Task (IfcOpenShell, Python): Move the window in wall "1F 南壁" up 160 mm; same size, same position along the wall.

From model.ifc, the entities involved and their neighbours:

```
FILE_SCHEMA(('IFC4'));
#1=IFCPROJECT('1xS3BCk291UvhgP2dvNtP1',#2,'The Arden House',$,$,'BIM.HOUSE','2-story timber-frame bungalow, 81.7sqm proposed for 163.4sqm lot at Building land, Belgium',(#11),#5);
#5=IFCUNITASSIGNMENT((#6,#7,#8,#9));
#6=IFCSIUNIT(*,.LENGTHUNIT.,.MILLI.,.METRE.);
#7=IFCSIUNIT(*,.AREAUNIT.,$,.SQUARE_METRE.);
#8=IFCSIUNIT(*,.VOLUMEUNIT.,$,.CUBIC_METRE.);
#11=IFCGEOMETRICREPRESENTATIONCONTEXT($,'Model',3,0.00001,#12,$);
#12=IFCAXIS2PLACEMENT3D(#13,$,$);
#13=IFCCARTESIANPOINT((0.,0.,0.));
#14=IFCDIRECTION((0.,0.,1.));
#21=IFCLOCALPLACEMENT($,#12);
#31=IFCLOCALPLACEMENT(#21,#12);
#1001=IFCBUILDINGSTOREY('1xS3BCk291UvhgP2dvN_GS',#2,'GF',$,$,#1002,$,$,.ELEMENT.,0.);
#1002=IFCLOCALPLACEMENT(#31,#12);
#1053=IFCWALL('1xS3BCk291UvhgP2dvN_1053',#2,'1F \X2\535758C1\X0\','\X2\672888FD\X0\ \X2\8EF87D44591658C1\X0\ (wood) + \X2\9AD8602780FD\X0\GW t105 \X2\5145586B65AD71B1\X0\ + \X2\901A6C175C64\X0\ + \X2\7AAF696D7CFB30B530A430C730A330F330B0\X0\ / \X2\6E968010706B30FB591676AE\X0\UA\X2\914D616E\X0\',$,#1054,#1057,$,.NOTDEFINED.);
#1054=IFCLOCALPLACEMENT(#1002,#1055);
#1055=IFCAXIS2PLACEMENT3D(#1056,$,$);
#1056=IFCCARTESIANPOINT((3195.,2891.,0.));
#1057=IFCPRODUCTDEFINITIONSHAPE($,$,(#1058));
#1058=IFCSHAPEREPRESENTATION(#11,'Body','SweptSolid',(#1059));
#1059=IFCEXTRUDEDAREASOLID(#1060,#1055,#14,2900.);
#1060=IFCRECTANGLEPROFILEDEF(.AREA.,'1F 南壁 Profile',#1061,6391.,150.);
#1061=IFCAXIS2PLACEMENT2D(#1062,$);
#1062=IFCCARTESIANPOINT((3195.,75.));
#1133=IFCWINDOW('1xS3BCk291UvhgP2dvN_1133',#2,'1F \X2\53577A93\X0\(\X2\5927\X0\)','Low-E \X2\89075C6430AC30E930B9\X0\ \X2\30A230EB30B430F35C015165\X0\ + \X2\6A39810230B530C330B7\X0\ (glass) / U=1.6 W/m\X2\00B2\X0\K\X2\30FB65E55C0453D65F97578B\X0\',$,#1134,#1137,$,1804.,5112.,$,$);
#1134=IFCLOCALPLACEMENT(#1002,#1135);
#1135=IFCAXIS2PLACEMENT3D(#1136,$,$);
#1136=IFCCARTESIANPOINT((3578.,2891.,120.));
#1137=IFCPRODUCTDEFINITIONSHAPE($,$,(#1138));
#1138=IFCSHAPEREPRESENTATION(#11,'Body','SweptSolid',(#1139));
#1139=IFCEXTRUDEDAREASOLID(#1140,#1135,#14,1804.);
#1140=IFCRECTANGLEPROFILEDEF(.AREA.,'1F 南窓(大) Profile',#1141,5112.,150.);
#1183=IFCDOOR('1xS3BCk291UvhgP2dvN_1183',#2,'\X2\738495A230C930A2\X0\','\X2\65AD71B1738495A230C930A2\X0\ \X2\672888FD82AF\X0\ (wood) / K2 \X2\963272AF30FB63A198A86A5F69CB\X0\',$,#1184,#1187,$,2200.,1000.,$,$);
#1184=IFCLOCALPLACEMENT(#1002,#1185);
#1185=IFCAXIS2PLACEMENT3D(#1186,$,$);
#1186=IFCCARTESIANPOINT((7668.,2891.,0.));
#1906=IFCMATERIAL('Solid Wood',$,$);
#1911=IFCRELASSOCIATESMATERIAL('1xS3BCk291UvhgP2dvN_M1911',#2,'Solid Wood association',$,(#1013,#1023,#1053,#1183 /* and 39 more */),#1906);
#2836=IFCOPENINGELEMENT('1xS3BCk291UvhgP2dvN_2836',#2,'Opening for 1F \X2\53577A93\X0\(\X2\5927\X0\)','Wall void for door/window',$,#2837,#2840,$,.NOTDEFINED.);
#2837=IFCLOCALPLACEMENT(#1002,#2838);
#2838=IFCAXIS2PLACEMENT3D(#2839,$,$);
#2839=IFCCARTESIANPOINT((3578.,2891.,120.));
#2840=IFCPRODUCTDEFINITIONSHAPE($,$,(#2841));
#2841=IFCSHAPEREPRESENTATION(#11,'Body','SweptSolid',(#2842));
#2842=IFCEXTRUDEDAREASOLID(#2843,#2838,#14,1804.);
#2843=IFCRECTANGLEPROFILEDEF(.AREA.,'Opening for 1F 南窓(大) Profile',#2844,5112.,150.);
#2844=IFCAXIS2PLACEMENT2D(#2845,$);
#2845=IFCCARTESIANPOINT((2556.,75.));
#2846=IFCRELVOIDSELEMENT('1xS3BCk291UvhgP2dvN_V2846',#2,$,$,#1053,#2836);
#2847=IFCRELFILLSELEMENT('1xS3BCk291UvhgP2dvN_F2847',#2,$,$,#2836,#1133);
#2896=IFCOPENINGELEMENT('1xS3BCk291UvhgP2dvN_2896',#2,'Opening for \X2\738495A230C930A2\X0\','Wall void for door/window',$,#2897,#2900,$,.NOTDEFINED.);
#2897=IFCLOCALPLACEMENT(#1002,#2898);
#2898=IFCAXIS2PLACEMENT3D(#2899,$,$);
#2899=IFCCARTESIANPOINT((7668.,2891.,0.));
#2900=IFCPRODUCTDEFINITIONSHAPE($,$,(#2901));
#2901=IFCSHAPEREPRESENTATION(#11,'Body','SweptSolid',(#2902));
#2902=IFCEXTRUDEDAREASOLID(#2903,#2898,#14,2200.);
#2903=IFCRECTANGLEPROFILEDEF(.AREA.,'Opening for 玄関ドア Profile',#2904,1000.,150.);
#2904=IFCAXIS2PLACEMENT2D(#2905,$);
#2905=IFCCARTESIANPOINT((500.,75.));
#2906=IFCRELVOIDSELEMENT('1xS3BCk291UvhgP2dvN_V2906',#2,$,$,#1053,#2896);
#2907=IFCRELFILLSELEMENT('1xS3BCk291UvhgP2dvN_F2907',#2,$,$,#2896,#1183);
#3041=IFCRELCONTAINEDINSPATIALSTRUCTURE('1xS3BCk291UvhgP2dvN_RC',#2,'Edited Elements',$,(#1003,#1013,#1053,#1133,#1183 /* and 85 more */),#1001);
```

```python
import numpy as np
import ifcopenshell
import ifcopenshell.api.geometry
import ifcopenshell.util.placement
import ifcopenshell.util.unit

model = ifcopenshell.open("model.ifc")
unit_scale = ifcopenshell.util.unit.calculate_unit_scale(model)

window = model.by_guid("1xS3BCk291UvhgP2dvN_1133")
opening = window.FillsVoids[0].RelatingOpeningElement
dz = 0.16 / unit_scale

shift = np.array([0.0, 0.0, dz])
# The window is not placed relative to its opening, so move both.
for product in (opening, window):
    matrix = ifcopenshell.util.placement.get_local_placement(product.ObjectPlacement)
    matrix[:3, 3] += shift
    ifcopenshell.api.geometry.edit_object_placement(model, product=product, matrix=matrix, is_si=False)

print(f"moved by {dz * unit_scale:+.3f} m")

model.write("model_updated.ifc")
```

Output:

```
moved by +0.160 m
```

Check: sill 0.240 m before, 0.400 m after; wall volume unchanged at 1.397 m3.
